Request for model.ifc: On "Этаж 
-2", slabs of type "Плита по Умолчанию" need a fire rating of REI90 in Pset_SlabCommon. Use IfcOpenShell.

First a look at what the model holds.

```python
import ifcopenshell
import ifcopenshell.util.element

model = ifcopenshell.open("model.ifc")
print(model.schema)
storey = next(s for s in model.by_type("IfcBuildingStorey") if s.Name == 'Этаж \r\n-2')
slabs = [e for e in ifcopenshell.util.element.get_decomposition(storey) if e.is_a("IfcSlab")]
seen = {}
for e in slabs:
    element_type = ifcopenshell.util.element.get_type(e)
    key = (element_type.Name if element_type != e and element_type else None, ifcopenshell.util.element.get_pset(e, "Pset_SlabCommon", "FireRating"))
    seen[key] = seen.get(key, 0) + 1
for (name, value), count in sorted(seen.items(), key=str):
    print(count, "x", name, "|", value)
```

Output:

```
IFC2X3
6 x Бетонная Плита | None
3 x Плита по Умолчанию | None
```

```python
import ifcopenshell
import ifcopenshell.api.pset
import ifcopenshell.util.element

model = ifcopenshell.open("model.ifc")

storey = next(s for s in model.by_type("IfcBuildingStorey") if s.Name == 'Этаж \r\n-2')
slabs = [e for e in ifcopenshell.util.element.get_decomposition(storey) if e.is_a("IfcSlab")]

count = 0
for e in slabs:
    element_type = ifcopenshell.util.element.get_type(e)
    if element_type in (None, e) or element_type.Name != "Плита по Умолчанию":
        continue
    # add_pset returns the element's existing set when there is one.
    pset = ifcopenshell.api.pset.add_pset(model, product=e, name="Pset_SlabCommon")
    ifcopenshell.api.pset.edit_pset(model, pset=pset, properties={"FireRating": "REI90"})
    count += 1

print(count, "slabs updated")

model.write("model_edited.ifc")
```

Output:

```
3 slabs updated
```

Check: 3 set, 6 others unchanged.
